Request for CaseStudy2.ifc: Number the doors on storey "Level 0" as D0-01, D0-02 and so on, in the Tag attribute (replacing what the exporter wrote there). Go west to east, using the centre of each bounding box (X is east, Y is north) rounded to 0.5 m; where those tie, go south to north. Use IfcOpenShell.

First a look at what the model holds.

```python
import ifcopenshell
import ifcopenshell.util.element
import ifcopenshell.util.placement

model = ifcopenshell.open("CaseStudy2.ifc")
print(model.schema)
storey = next(s for s in model.by_type("IfcBuildingStorey") if s.Name == "Level 0")
doors = [e for e in ifcopenshell.util.element.get_decomposition(storey) if e.is_a("IfcDoor")]
for e in sorted(doors, key=lambda e: e.id()):
    origin = ifcopenshell.util.placement.get_local_placement(e.ObjectPlacement)[:3, 3]
    print(e.id(), e.Tag, e.Name, origin.round(2) + 0.0, sep=" | ")
```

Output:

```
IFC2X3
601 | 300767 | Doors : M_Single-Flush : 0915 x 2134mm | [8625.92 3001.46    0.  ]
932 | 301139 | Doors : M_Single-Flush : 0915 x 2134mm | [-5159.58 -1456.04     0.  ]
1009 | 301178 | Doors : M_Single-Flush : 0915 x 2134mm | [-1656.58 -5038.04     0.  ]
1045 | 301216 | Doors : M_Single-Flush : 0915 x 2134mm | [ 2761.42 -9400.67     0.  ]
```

```python
import ifcopenshell
import ifcopenshell.geom
import ifcopenshell.util.element
import ifcopenshell.util.shape

model = ifcopenshell.open("CaseStudy2.ifc")
settings = ifcopenshell.geom.settings()
settings.set("use-world-coords", True)


def centre(element):
    shape = ifcopenshell.geom.create_shape(settings, element)
    return ifcopenshell.util.shape.get_bbox_centroid(shape.geometry)


storey = next(s for s in model.by_type("IfcBuildingStorey") if s.Name == "Level 0")
doors = [e for e in ifcopenshell.util.element.get_decomposition(storey) if e.is_a("IfcDoor")]

# Insertion points can sit at a corner or the storey origin, so sort by the geometry (in metres).
centres = {e: centre(e) for e in doors}
doors.sort(key=lambda e: (round(centres[e][0] / 0.5), centres[e][1]))

for i, e in enumerate(doors, start=1):
    number = f"D0-{i:02d}"
    e.Tag = number
    print(e.id(), number)

model.write("CaseStudy2_v2.ifc")
```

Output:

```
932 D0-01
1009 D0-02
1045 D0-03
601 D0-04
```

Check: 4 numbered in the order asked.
